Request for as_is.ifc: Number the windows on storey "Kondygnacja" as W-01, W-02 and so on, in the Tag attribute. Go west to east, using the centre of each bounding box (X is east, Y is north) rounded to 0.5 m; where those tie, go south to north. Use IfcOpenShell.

First a look at what the model holds.

```python
import ifcopenshell
import ifcopenshell.util.element
import ifcopenshell.util.placement

model = ifcopenshell.open("as_is.ifc")
print(model.schema)
storey = next(s for s in model.by_type("IfcBuildingStorey") if s.Name == "Kondygnacja")
windows = [e for e in ifcopenshell.util.element.get_decomposition(storey) if e.is_a("IfcWindow")]
for e in sorted(windows, key=lambda e: e.id()):
    origin = ifcopenshell.util.placement.get_local_placement(e.ObjectPlacement)[:3, 3]
    print(e.id(), e.Tag, e.Name, origin.round(2) + 0.0, sep=" | ")
```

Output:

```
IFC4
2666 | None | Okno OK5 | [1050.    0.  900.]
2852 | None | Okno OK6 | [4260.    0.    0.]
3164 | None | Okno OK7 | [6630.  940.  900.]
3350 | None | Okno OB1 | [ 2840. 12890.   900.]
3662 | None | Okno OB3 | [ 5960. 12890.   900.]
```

```python
import ifcopenshell
import ifcopenshell.geom
import ifcopenshell.util.element
import ifcopenshell.util.shape

model = ifcopenshell.open("as_is.ifc")
settings = ifcopenshell.geom.settings()
settings.set("use-world-coords", True)


def centre(element):
    shape = ifcopenshell.geom.create_shape(settings, element)
    return ifcopenshell.util.shape.get_bbox_centroid(shape.geometry)


storey = next(s for s in model.by_type("IfcBuildingStorey") if s.Name == "Kondygnacja")
windows = [e for e in ifcopenshell.util.element.get_decomposition(storey) if e.is_a("IfcWindow")]

# Insertion points can sit at a corner or the storey origin, so sort by the geometry (in metres).
centres = {e: centre(e) for e in windows}
windows.sort(key=lambda e: (round(centres[e][0] / 0.5), centres[e][1]))

for i, e in enumerate(windows, start=1):
    number = f"W-{i:02d}"
    e.Tag = number
    print(e.id(), number)

model.write("as_is_edited.ifc")
```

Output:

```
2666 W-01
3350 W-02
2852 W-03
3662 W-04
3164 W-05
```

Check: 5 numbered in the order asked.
